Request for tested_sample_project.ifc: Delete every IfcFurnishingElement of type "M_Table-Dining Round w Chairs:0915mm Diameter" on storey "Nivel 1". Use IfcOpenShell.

First a look at what the model holds.

```python
import ifcopenshell
import ifcopenshell.util.element

model = ifcopenshell.open("tested_sample_project.ifc")
print(model.schema)
storey = next(s for s in model.by_type("IfcBuildingStorey") if s.Name == "Nivel 1")
furniture = [e for e in ifcopenshell.util.element.get_decomposition(storey) if e.is_a("IfcFurnishingElement")]
seen = {}
for e in furniture:
    element_type = ifcopenshell.util.element.get_type(e)
    name = element_type.Name if element_type not in (None, e) else None
    seen[name] = seen.get(name, 0) + 1
for name, count in sorted(seen.items(), key=str):
    print(count, "x", name)
```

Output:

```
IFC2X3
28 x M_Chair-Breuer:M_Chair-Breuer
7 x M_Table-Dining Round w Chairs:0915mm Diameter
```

```python
import ifcopenshell
import ifcopenshell.api.root
import ifcopenshell.util.element

model = ifcopenshell.open("tested_sample_project.ifc")

storey = next(s for s in model.by_type("IfcBuildingStorey") if s.Name == "Nivel 1")
furniture = [e for e in ifcopenshell.util.element.get_decomposition(storey) if e.is_a("IfcFurnishingElement")]
targets = [e for e in furniture if (t := ifcopenshell.util.element.get_type(e)) not in (None, e) and t.Name == "M_Table-Dining Round w Chairs:0915mm Diameter"]

for e in targets:
    ifcopenshell.api.root.remove_product(model, product=e)
print(len(targets), "removed")

model.write("tested_sample_project_v2.ifc")
```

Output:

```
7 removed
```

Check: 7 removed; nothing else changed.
